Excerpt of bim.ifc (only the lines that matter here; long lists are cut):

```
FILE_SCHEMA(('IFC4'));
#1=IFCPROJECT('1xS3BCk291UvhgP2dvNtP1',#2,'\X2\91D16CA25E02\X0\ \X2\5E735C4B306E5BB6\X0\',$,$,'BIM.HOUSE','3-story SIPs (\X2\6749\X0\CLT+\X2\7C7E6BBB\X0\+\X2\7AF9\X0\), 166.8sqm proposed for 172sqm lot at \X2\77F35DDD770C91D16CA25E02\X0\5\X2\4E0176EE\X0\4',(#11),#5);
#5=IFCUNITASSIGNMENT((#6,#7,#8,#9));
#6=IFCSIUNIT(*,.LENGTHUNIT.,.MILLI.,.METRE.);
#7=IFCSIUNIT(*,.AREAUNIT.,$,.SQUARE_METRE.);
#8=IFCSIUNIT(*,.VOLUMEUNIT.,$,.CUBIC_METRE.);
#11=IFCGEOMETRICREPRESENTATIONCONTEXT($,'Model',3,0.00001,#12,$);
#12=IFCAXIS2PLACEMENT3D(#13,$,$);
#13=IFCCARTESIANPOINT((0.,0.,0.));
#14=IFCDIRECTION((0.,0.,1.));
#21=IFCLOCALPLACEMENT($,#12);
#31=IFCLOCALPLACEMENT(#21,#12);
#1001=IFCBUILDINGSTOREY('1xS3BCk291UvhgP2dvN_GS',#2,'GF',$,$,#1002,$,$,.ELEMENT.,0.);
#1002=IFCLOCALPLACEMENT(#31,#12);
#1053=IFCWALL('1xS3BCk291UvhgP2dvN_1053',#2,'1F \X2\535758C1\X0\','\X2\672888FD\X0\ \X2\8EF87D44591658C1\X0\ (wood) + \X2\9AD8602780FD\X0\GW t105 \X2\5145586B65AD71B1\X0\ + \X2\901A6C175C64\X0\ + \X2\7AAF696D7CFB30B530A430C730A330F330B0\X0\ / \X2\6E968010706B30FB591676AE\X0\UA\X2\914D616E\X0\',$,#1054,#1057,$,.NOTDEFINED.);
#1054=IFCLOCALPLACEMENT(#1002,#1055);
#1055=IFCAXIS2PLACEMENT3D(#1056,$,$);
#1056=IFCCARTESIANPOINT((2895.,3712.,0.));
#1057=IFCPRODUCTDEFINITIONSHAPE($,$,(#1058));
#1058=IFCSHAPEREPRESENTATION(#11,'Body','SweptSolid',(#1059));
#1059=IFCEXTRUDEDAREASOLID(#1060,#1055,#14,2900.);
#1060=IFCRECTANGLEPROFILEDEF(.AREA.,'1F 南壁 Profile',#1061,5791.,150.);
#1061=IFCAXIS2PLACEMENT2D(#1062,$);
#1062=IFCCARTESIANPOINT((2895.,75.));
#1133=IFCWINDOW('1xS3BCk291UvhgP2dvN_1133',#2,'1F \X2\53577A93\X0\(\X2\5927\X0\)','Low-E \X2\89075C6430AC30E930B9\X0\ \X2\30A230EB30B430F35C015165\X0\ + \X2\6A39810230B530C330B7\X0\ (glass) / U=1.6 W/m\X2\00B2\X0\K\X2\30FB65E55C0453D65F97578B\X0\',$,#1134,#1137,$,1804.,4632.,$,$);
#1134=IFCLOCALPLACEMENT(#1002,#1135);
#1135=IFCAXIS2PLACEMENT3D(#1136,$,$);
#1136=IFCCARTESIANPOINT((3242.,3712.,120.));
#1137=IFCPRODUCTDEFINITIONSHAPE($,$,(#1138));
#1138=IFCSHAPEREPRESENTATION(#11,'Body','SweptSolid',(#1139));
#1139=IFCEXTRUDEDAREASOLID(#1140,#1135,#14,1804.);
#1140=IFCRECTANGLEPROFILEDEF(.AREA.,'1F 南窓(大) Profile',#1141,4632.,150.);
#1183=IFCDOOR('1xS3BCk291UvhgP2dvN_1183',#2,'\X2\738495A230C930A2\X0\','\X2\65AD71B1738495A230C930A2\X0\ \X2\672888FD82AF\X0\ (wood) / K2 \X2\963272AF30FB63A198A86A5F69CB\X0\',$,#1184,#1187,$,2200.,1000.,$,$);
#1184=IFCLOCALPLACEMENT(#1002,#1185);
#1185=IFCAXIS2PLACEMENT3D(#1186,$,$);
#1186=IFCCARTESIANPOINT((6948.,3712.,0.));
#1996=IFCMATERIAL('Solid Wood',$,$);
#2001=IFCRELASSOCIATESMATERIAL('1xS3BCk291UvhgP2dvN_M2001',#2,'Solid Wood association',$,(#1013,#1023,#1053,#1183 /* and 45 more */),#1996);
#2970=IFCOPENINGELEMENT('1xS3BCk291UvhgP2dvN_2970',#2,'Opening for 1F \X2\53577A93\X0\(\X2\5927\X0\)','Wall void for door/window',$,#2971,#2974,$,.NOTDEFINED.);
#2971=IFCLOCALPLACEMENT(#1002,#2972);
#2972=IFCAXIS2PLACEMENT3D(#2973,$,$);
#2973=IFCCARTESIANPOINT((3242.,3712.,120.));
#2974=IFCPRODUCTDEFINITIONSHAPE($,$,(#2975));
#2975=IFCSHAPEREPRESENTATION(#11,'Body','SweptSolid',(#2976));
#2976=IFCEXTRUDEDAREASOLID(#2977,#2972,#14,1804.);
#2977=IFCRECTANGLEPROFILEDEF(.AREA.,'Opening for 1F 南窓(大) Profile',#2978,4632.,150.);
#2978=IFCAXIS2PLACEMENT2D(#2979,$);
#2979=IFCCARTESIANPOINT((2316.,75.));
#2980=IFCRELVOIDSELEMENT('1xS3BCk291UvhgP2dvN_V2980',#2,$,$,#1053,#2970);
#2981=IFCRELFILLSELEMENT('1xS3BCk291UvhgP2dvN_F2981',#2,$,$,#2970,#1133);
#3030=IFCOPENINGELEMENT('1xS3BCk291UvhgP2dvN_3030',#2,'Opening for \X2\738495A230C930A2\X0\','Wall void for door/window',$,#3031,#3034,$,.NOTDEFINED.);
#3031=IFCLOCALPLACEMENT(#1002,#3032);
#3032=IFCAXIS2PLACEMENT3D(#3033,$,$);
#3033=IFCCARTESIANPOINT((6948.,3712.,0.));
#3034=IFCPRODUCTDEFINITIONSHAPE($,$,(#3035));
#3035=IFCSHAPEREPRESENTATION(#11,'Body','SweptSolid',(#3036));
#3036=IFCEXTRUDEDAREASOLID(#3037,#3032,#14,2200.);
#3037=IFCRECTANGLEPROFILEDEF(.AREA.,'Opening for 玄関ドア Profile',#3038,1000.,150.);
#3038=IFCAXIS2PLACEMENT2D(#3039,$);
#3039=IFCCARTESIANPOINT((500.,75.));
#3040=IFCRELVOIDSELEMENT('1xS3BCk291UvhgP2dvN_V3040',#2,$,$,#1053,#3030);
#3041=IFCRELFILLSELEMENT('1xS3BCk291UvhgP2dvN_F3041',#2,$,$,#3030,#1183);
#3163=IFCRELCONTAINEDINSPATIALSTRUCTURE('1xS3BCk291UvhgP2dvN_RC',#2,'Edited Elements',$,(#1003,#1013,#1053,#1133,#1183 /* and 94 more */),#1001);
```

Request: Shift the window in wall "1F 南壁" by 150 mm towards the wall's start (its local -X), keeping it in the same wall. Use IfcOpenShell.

```python
import ifcopenshell
import ifcopenshell.api.geometry
import ifcopenshell.util.placement
import ifcopenshell.util.unit

model = ifcopenshell.open("bim.ifc")
unit_scale = ifcopenshell.util.unit.calculate_unit_scale(model)

window = model.by_guid("1xS3BCk291UvhgP2dvN_1133")
opening = window.FillsVoids[0].RelatingOpeningElement
wall = opening.VoidsElements[0].RelatingBuildingElement

wall_matrix = ifcopenshell.util.placement.get_local_placement(wall.ObjectPlacement)
shift = wall_matrix[:3, 0] * -0.15 / unit_scale
before = ifcopenshell.util.placement.get_local_placement(window.ObjectPlacement)[:3, 3].copy()

# The window is not placed relative to its opening, so move both.
for product in (opening, window):
    matrix = ifcopenshell.util.placement.get_local_placement(product.ObjectPlacement)
    matrix[:3, 3] += shift
    ifcopenshell.api.geometry.edit_object_placement(model, product=product, matrix=matrix, is_si=False)

after = ifcopenshell.util.placement.get_local_placement(window.ObjectPlacement)[:3, 3]
print("window moved by", (after - before).round(3) + 0.0)

model.write("bim-out.ifc")
```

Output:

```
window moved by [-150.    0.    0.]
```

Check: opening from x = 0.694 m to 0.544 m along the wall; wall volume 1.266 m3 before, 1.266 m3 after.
